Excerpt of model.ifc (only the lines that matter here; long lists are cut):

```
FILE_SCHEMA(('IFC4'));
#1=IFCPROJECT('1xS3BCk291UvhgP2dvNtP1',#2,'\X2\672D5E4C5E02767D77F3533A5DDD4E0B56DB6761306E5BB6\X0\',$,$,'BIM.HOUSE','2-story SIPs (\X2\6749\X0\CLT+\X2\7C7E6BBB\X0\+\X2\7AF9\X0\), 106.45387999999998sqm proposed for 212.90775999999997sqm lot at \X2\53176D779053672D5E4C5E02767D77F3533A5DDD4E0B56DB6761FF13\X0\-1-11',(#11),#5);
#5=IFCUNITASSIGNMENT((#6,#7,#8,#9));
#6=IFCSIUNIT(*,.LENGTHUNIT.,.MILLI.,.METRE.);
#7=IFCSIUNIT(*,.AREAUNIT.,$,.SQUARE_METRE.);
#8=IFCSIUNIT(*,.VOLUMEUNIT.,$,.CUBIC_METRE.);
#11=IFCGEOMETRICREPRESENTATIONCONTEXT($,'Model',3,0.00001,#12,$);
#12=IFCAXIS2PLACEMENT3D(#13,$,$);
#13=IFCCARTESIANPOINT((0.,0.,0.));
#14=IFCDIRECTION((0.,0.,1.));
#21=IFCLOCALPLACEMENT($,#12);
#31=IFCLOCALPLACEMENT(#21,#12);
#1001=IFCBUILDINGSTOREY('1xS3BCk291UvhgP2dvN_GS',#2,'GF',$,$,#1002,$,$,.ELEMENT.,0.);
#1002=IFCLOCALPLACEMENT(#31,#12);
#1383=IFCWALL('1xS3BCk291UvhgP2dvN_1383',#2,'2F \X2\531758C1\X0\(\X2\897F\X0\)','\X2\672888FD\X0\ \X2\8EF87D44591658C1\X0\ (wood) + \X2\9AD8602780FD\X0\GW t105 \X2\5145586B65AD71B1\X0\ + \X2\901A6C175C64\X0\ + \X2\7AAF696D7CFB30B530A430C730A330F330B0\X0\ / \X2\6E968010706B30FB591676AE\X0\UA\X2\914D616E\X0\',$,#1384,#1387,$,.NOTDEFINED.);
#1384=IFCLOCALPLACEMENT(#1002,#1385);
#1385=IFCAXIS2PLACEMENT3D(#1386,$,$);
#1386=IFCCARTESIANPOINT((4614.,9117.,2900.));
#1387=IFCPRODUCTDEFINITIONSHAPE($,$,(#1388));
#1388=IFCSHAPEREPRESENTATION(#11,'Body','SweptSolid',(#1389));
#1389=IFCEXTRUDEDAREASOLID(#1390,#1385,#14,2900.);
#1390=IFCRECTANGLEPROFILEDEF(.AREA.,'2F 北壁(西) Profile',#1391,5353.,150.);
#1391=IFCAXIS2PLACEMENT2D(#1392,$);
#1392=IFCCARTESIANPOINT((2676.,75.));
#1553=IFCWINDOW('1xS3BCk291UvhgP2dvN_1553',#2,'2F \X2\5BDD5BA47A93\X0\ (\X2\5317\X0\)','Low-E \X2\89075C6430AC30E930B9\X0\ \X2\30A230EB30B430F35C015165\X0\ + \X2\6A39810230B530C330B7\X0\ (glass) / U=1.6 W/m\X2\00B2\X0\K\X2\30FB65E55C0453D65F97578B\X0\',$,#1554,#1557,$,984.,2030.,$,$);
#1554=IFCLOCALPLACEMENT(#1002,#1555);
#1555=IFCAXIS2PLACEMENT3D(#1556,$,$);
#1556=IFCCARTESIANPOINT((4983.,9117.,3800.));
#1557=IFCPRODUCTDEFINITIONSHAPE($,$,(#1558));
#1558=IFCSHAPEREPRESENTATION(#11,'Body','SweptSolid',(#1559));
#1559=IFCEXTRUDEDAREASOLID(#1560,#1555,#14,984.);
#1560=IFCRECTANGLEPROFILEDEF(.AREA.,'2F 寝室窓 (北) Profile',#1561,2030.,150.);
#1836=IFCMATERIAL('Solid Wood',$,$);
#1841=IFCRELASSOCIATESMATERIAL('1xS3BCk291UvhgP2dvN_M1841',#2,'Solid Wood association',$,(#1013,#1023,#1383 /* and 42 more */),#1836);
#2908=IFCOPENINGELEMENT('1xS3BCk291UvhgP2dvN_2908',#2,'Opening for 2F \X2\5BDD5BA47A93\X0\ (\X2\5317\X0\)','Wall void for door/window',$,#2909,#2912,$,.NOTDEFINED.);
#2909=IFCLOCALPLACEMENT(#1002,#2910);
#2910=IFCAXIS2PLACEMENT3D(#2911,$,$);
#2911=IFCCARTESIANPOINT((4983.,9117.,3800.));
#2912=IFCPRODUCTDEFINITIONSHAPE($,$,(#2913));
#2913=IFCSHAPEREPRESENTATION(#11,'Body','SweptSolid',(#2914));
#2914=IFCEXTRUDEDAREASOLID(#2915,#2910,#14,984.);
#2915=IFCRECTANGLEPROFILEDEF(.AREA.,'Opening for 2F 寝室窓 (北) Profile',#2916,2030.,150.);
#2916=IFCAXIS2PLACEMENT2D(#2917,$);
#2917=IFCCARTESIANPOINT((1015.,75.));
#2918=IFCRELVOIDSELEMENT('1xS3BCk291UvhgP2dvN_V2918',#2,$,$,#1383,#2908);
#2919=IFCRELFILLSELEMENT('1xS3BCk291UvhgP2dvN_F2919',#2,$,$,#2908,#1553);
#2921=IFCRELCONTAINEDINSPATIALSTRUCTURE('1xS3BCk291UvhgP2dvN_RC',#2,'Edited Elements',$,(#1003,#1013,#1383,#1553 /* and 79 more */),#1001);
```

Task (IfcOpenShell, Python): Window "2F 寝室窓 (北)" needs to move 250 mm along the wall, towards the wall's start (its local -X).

```python
import ifcopenshell
import ifcopenshell.api.geometry
import ifcopenshell.util.placement
import ifcopenshell.util.unit

model = ifcopenshell.open("model.ifc")
unit_scale = ifcopenshell.util.unit.calculate_unit_scale(model)

window = model.by_id(1553)
opening = window.FillsVoids[0].RelatingOpeningElement
wall = opening.VoidsElements[0].RelatingBuildingElement

wall_matrix = ifcopenshell.util.placement.get_local_placement(wall.ObjectPlacement)
shift = wall_matrix[:3, 0] * -0.25 / unit_scale
before = ifcopenshell.util.placement.get_local_placement(window.ObjectPlacement)[:3, 3].copy()

# The window is not placed relative to its opening, so move both.
for product in (opening, window):
    matrix = ifcopenshell.util.placement.get_local_placement(product.ObjectPlacement)
    matrix[:3, 3] += shift
    ifcopenshell.api.geometry.edit_object_placement(model, product=product, matrix=matrix, is_si=False)

after = ifcopenshell.util.placement.get_local_placement(window.ObjectPlacement)[:3, 3]
print("window moved by", (after - before).round(3) + 0.0)

model.write("model-out.ifc")
```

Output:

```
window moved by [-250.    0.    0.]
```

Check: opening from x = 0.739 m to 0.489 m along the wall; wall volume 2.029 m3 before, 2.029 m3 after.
